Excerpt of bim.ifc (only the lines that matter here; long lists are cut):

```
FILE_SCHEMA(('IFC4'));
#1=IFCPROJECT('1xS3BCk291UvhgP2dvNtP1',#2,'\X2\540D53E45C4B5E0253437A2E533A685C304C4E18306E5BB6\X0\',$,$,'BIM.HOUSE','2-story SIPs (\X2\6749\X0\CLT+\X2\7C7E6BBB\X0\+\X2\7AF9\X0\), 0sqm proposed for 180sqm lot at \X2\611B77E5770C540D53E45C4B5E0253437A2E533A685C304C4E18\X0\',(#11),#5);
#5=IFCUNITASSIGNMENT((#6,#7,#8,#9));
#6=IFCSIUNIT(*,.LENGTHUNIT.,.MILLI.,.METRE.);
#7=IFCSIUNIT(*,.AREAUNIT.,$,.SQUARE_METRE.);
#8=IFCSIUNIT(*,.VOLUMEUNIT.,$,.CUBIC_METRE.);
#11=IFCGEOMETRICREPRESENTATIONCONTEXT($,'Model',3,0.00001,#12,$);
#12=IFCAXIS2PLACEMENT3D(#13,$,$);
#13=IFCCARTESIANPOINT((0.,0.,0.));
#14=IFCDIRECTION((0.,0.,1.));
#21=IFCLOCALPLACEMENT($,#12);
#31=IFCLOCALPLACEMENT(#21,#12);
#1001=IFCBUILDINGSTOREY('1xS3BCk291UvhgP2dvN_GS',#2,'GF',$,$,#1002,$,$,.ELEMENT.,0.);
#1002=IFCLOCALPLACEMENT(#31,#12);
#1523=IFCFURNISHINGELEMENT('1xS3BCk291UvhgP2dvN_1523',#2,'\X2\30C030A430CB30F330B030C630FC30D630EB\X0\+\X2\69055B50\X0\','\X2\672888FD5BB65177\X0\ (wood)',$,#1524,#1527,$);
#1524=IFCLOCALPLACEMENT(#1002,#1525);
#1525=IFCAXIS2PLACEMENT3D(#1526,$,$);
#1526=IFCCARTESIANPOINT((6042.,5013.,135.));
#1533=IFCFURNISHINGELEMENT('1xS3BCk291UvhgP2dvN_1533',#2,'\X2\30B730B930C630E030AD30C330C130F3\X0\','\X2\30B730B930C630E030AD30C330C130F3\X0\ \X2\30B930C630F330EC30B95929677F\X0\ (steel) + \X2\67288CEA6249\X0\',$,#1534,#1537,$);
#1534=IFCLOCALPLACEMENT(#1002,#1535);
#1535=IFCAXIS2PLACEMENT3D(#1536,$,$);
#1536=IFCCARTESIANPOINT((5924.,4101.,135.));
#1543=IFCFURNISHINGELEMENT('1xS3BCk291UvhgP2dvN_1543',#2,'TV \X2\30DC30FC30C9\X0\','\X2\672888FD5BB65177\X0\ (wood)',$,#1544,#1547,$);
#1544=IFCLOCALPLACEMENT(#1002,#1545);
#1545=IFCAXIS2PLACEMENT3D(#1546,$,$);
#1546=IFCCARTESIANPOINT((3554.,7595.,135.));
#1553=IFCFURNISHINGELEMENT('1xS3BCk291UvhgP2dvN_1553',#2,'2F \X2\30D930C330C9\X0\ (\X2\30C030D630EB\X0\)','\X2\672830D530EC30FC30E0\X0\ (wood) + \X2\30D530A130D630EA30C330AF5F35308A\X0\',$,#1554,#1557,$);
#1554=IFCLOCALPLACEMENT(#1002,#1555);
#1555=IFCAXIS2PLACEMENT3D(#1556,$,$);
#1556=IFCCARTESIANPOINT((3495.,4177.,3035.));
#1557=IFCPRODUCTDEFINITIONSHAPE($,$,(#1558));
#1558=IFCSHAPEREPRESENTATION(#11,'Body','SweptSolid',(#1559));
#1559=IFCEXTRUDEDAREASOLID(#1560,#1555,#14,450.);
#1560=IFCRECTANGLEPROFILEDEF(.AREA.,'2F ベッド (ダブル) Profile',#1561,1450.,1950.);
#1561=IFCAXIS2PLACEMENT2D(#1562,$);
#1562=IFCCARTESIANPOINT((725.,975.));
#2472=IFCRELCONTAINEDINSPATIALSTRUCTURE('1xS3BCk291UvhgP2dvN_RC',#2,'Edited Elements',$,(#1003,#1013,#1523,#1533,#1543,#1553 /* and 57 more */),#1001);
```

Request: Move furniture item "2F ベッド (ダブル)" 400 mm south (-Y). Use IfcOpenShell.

```python
import ifcopenshell
import ifcopenshell.api.geometry
import ifcopenshell.util.placement

model = ifcopenshell.open("bim.ifc")

item = model.by_guid("1xS3BCk291UvhgP2dvN_1553")
matrix = ifcopenshell.util.placement.get_local_placement(item.ObjectPlacement)
matrix[1, 3] -= 400.0
ifcopenshell.api.geometry.edit_object_placement(model, product=item, matrix=matrix, is_si=False)

print(ifcopenshell.util.placement.get_local_placement(item.ObjectPlacement).round(3) + 0.0)

model.write("bim_edited.ifc")
```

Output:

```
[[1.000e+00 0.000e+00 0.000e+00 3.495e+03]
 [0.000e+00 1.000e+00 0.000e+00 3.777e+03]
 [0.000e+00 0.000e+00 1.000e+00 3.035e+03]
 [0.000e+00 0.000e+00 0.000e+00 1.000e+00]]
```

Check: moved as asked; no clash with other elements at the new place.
